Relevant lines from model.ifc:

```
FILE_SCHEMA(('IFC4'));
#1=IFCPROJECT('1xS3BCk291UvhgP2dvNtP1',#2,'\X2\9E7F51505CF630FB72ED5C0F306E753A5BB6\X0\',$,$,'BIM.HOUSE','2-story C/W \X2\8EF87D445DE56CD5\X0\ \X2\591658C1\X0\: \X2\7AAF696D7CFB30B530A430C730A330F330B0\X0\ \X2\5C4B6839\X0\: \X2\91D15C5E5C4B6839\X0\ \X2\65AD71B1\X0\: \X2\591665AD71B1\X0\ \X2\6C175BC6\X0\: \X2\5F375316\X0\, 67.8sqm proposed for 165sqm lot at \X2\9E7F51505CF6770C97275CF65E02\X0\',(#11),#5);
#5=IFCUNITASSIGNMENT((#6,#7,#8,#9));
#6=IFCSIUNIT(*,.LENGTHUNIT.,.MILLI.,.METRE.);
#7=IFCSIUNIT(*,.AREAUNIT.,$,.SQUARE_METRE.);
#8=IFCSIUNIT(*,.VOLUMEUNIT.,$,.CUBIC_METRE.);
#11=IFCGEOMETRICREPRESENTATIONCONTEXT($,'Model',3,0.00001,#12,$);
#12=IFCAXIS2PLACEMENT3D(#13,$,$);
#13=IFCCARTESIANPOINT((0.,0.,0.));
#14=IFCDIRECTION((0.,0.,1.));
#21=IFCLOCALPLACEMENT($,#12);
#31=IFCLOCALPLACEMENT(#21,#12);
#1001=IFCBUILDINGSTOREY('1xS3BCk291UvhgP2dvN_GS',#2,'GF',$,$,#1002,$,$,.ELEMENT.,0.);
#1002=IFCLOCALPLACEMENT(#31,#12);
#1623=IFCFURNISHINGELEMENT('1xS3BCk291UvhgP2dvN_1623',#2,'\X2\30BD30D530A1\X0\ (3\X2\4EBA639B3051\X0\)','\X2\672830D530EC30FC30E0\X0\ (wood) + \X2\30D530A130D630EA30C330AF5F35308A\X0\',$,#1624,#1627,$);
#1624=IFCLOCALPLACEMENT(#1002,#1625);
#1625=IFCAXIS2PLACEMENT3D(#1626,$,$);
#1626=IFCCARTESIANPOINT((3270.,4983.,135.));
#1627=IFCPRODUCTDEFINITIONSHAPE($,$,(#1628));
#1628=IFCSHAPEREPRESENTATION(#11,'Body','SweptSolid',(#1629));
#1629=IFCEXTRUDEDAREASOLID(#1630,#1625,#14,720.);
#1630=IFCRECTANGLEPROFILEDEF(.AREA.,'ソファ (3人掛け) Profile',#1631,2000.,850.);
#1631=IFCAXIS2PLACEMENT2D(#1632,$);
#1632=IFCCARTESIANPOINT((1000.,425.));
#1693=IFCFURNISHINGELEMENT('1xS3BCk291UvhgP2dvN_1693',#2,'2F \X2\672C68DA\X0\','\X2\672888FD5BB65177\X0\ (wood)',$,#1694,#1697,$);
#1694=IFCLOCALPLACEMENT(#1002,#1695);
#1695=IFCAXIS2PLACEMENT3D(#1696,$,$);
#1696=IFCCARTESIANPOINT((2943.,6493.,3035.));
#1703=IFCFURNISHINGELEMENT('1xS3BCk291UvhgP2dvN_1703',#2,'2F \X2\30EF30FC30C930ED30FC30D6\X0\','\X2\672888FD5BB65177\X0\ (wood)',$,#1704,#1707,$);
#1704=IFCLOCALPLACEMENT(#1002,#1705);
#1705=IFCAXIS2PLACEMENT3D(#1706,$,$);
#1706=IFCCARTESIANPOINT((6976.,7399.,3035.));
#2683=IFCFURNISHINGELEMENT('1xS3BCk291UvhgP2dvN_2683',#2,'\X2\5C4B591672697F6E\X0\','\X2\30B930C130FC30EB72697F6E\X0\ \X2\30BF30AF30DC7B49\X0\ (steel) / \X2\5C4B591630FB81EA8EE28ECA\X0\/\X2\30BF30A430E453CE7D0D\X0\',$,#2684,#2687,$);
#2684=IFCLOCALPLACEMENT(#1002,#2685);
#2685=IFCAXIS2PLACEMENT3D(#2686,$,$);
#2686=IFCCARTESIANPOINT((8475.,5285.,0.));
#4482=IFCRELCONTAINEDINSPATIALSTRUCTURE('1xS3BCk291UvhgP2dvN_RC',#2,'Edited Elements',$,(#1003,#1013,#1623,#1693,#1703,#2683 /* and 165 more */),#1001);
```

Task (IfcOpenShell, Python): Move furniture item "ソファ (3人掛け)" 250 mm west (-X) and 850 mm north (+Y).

```python
import ifcopenshell
import ifcopenshell.api.geometry
import ifcopenshell.util.placement

model = ifcopenshell.open("model.ifc")

item = model.by_id(1623)
matrix = ifcopenshell.util.placement.get_local_placement(item.ObjectPlacement)
matrix[0, 3] -= 250.0
matrix[1, 3] += 850.0
ifcopenshell.api.geometry.edit_object_placement(model, product=item, matrix=matrix, is_si=False)

print(ifcopenshell.util.placement.get_local_placement(item.ObjectPlacement).round(3) + 0.0)

model.write("model_rev.ifc")
```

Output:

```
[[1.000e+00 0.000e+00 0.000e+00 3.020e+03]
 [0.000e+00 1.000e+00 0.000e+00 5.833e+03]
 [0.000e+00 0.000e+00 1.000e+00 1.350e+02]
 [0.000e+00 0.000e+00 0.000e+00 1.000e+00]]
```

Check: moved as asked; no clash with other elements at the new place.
